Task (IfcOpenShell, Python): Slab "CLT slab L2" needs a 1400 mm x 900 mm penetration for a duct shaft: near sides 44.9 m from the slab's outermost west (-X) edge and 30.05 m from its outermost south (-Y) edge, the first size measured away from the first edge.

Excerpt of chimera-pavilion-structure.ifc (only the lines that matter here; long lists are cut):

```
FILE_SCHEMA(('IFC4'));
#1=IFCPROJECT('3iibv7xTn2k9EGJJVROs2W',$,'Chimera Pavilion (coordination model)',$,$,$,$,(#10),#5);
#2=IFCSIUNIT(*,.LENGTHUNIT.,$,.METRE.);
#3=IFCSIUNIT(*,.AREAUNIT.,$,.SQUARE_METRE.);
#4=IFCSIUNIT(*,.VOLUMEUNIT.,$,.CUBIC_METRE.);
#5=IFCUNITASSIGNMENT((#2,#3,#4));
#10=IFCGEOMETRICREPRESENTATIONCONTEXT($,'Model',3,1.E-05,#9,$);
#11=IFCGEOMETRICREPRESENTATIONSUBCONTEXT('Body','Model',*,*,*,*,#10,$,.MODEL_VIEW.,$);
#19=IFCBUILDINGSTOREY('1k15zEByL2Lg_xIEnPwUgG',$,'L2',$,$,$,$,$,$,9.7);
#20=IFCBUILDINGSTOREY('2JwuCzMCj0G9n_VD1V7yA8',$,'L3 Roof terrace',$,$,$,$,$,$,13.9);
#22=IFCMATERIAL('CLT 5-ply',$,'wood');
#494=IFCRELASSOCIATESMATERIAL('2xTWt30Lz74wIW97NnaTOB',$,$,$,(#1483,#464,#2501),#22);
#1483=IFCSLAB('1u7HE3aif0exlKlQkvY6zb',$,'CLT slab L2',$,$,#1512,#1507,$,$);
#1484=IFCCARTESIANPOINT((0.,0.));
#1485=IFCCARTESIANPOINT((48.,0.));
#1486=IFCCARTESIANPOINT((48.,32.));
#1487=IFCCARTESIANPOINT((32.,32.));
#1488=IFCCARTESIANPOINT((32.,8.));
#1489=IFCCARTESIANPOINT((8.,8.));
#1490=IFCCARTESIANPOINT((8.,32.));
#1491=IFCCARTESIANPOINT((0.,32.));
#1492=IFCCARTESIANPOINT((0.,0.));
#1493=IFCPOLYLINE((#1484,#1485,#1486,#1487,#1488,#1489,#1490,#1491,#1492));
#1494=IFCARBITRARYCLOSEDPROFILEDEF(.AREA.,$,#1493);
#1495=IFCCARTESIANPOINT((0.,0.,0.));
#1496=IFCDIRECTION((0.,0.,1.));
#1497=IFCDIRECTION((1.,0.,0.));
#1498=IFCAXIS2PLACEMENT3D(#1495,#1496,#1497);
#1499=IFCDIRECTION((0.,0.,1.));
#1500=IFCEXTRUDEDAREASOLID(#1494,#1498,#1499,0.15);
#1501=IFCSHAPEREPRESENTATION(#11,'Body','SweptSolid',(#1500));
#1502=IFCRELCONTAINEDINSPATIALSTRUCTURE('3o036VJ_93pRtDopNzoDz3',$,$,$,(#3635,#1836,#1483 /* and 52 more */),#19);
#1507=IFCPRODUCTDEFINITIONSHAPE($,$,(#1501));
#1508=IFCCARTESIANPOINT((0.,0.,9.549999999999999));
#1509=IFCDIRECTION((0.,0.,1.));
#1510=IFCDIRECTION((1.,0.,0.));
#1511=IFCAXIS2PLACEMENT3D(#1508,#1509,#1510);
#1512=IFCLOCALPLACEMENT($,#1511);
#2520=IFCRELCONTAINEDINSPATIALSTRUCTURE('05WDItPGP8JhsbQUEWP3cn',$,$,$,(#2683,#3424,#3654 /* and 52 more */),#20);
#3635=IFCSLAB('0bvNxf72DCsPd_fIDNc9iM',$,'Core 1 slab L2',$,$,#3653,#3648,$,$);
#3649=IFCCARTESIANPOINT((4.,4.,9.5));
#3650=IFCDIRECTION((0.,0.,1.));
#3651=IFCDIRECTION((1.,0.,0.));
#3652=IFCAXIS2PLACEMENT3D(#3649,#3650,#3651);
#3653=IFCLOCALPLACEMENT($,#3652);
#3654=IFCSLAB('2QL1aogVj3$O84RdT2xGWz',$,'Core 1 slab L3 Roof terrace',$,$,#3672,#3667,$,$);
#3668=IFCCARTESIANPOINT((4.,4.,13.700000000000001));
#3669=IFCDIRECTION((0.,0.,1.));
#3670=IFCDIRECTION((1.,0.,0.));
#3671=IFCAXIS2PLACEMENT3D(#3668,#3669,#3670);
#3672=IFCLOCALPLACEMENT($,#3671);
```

```python
import numpy as np
import ifcopenshell
import ifcopenshell.api.feature
import ifcopenshell.api.geometry
import ifcopenshell.api.root
import ifcopenshell.geom
import ifcopenshell.util.placement
import ifcopenshell.util.representation
import ifcopenshell.util.shape
import ifcopenshell.util.unit

model = ifcopenshell.open("chimera-pavilion-structure.ifc")
unit_scale = ifcopenshell.util.unit.calculate_unit_scale(model)
settings = ifcopenshell.geom.settings()


def volume(element):
    """Net volume in cubic metres, openings subtracted."""
    shape = ifcopenshell.geom.create_shape(settings, element)
    return ifcopenshell.util.shape.get_volume(shape.geometry)


slab = model.by_guid("1u7HE3aif0exlKlQkvY6zb")
before = volume(slab)

# Extent in the slab's own axes, in metres. The edges named are its -X and -Y sides.
slab_shape = ifcopenshell.geom.create_shape(settings, slab)
vertices = ifcopenshell.util.shape.get_vertices(slab_shape.geometry)
x_min, y_min, bottom = vertices.min(axis=0)
top = vertices[:, 2].max()

opening = ifcopenshell.api.root.create_entity(model, ifc_class="IfcOpeningElement", name="Duct shaft opening", predefined_type="OPENING")
context = ifcopenshell.util.representation.get_context(model, "Model", "Body", "MODEL_VIEW")
width, depth = 1.4, 0.9
outline = [(0.0, 0.0), (width, 0.0), (width, depth), (0.0, depth), (0.0, 0.0)]
# Overshoot both faces by 50 mm so the cut is clean.
shape = ifcopenshell.api.geometry.add_slab_representation(
    model, context=context, depth=top - bottom + 0.1, polyline=outline
)
ifcopenshell.api.geometry.assign_representation(model, product=opening, representation=shape)

matrix = ifcopenshell.util.placement.get_local_placement(slab.ObjectPlacement)
matrix[:, 3] = matrix @ np.append(np.array([x_min + 44.9, y_min + 30.05, bottom - 0.05]) / unit_scale, 1.0)
ifcopenshell.api.geometry.edit_object_placement(model, product=opening, matrix=matrix, is_si=False)
ifcopenshell.api.feature.add_feature(model, feature=opening, element=slab)

after = volume(slab)

print(f"slab volume {before:.3f} -> {after:.3f} m3")

model.write("chimera-pavilion-structure_rev.ifc")
```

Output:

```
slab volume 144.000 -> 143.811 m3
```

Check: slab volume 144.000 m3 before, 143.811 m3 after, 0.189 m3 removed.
